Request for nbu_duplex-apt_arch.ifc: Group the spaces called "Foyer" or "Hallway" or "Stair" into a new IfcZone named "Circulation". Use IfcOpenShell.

First a look at what the model holds.

```python
import ifcopenshell

model = ifcopenshell.open("nbu_duplex-apt_arch.ifc")
print(model.schema)
seen = {}
for space in model.by_type("IfcSpace"):
    seen[space.LongName] = seen.get(space.LongName, 0) + 1
for name, count in sorted(seen.items(), key=str):
    print(count, "x", name)
print("zones:", [z.Name for z in model.by_type("IfcZone")][:20])
```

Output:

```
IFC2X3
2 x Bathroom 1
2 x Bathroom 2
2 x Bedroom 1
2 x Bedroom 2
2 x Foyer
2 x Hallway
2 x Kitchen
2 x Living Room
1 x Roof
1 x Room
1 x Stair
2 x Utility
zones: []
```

```python
import ifcopenshell
import ifcopenshell.api.group
import ifcopenshell.api.root

model = ifcopenshell.open("nbu_duplex-apt_arch.ifc")

names = {"Foyer", "Hallway", "Stair"}
spaces = [s for s in model.by_type("IfcSpace") if s.LongName in names]

zone = ifcopenshell.api.root.create_entity(model, ifc_class="IfcZone", name="Circulation")
ifcopenshell.api.group.assign_group(model, products=spaces, group=zone)
print(len(spaces), "spaces in", zone.Name)

model.write("nbu_duplex-apt_arch_updated.ifc")
```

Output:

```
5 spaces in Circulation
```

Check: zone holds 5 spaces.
